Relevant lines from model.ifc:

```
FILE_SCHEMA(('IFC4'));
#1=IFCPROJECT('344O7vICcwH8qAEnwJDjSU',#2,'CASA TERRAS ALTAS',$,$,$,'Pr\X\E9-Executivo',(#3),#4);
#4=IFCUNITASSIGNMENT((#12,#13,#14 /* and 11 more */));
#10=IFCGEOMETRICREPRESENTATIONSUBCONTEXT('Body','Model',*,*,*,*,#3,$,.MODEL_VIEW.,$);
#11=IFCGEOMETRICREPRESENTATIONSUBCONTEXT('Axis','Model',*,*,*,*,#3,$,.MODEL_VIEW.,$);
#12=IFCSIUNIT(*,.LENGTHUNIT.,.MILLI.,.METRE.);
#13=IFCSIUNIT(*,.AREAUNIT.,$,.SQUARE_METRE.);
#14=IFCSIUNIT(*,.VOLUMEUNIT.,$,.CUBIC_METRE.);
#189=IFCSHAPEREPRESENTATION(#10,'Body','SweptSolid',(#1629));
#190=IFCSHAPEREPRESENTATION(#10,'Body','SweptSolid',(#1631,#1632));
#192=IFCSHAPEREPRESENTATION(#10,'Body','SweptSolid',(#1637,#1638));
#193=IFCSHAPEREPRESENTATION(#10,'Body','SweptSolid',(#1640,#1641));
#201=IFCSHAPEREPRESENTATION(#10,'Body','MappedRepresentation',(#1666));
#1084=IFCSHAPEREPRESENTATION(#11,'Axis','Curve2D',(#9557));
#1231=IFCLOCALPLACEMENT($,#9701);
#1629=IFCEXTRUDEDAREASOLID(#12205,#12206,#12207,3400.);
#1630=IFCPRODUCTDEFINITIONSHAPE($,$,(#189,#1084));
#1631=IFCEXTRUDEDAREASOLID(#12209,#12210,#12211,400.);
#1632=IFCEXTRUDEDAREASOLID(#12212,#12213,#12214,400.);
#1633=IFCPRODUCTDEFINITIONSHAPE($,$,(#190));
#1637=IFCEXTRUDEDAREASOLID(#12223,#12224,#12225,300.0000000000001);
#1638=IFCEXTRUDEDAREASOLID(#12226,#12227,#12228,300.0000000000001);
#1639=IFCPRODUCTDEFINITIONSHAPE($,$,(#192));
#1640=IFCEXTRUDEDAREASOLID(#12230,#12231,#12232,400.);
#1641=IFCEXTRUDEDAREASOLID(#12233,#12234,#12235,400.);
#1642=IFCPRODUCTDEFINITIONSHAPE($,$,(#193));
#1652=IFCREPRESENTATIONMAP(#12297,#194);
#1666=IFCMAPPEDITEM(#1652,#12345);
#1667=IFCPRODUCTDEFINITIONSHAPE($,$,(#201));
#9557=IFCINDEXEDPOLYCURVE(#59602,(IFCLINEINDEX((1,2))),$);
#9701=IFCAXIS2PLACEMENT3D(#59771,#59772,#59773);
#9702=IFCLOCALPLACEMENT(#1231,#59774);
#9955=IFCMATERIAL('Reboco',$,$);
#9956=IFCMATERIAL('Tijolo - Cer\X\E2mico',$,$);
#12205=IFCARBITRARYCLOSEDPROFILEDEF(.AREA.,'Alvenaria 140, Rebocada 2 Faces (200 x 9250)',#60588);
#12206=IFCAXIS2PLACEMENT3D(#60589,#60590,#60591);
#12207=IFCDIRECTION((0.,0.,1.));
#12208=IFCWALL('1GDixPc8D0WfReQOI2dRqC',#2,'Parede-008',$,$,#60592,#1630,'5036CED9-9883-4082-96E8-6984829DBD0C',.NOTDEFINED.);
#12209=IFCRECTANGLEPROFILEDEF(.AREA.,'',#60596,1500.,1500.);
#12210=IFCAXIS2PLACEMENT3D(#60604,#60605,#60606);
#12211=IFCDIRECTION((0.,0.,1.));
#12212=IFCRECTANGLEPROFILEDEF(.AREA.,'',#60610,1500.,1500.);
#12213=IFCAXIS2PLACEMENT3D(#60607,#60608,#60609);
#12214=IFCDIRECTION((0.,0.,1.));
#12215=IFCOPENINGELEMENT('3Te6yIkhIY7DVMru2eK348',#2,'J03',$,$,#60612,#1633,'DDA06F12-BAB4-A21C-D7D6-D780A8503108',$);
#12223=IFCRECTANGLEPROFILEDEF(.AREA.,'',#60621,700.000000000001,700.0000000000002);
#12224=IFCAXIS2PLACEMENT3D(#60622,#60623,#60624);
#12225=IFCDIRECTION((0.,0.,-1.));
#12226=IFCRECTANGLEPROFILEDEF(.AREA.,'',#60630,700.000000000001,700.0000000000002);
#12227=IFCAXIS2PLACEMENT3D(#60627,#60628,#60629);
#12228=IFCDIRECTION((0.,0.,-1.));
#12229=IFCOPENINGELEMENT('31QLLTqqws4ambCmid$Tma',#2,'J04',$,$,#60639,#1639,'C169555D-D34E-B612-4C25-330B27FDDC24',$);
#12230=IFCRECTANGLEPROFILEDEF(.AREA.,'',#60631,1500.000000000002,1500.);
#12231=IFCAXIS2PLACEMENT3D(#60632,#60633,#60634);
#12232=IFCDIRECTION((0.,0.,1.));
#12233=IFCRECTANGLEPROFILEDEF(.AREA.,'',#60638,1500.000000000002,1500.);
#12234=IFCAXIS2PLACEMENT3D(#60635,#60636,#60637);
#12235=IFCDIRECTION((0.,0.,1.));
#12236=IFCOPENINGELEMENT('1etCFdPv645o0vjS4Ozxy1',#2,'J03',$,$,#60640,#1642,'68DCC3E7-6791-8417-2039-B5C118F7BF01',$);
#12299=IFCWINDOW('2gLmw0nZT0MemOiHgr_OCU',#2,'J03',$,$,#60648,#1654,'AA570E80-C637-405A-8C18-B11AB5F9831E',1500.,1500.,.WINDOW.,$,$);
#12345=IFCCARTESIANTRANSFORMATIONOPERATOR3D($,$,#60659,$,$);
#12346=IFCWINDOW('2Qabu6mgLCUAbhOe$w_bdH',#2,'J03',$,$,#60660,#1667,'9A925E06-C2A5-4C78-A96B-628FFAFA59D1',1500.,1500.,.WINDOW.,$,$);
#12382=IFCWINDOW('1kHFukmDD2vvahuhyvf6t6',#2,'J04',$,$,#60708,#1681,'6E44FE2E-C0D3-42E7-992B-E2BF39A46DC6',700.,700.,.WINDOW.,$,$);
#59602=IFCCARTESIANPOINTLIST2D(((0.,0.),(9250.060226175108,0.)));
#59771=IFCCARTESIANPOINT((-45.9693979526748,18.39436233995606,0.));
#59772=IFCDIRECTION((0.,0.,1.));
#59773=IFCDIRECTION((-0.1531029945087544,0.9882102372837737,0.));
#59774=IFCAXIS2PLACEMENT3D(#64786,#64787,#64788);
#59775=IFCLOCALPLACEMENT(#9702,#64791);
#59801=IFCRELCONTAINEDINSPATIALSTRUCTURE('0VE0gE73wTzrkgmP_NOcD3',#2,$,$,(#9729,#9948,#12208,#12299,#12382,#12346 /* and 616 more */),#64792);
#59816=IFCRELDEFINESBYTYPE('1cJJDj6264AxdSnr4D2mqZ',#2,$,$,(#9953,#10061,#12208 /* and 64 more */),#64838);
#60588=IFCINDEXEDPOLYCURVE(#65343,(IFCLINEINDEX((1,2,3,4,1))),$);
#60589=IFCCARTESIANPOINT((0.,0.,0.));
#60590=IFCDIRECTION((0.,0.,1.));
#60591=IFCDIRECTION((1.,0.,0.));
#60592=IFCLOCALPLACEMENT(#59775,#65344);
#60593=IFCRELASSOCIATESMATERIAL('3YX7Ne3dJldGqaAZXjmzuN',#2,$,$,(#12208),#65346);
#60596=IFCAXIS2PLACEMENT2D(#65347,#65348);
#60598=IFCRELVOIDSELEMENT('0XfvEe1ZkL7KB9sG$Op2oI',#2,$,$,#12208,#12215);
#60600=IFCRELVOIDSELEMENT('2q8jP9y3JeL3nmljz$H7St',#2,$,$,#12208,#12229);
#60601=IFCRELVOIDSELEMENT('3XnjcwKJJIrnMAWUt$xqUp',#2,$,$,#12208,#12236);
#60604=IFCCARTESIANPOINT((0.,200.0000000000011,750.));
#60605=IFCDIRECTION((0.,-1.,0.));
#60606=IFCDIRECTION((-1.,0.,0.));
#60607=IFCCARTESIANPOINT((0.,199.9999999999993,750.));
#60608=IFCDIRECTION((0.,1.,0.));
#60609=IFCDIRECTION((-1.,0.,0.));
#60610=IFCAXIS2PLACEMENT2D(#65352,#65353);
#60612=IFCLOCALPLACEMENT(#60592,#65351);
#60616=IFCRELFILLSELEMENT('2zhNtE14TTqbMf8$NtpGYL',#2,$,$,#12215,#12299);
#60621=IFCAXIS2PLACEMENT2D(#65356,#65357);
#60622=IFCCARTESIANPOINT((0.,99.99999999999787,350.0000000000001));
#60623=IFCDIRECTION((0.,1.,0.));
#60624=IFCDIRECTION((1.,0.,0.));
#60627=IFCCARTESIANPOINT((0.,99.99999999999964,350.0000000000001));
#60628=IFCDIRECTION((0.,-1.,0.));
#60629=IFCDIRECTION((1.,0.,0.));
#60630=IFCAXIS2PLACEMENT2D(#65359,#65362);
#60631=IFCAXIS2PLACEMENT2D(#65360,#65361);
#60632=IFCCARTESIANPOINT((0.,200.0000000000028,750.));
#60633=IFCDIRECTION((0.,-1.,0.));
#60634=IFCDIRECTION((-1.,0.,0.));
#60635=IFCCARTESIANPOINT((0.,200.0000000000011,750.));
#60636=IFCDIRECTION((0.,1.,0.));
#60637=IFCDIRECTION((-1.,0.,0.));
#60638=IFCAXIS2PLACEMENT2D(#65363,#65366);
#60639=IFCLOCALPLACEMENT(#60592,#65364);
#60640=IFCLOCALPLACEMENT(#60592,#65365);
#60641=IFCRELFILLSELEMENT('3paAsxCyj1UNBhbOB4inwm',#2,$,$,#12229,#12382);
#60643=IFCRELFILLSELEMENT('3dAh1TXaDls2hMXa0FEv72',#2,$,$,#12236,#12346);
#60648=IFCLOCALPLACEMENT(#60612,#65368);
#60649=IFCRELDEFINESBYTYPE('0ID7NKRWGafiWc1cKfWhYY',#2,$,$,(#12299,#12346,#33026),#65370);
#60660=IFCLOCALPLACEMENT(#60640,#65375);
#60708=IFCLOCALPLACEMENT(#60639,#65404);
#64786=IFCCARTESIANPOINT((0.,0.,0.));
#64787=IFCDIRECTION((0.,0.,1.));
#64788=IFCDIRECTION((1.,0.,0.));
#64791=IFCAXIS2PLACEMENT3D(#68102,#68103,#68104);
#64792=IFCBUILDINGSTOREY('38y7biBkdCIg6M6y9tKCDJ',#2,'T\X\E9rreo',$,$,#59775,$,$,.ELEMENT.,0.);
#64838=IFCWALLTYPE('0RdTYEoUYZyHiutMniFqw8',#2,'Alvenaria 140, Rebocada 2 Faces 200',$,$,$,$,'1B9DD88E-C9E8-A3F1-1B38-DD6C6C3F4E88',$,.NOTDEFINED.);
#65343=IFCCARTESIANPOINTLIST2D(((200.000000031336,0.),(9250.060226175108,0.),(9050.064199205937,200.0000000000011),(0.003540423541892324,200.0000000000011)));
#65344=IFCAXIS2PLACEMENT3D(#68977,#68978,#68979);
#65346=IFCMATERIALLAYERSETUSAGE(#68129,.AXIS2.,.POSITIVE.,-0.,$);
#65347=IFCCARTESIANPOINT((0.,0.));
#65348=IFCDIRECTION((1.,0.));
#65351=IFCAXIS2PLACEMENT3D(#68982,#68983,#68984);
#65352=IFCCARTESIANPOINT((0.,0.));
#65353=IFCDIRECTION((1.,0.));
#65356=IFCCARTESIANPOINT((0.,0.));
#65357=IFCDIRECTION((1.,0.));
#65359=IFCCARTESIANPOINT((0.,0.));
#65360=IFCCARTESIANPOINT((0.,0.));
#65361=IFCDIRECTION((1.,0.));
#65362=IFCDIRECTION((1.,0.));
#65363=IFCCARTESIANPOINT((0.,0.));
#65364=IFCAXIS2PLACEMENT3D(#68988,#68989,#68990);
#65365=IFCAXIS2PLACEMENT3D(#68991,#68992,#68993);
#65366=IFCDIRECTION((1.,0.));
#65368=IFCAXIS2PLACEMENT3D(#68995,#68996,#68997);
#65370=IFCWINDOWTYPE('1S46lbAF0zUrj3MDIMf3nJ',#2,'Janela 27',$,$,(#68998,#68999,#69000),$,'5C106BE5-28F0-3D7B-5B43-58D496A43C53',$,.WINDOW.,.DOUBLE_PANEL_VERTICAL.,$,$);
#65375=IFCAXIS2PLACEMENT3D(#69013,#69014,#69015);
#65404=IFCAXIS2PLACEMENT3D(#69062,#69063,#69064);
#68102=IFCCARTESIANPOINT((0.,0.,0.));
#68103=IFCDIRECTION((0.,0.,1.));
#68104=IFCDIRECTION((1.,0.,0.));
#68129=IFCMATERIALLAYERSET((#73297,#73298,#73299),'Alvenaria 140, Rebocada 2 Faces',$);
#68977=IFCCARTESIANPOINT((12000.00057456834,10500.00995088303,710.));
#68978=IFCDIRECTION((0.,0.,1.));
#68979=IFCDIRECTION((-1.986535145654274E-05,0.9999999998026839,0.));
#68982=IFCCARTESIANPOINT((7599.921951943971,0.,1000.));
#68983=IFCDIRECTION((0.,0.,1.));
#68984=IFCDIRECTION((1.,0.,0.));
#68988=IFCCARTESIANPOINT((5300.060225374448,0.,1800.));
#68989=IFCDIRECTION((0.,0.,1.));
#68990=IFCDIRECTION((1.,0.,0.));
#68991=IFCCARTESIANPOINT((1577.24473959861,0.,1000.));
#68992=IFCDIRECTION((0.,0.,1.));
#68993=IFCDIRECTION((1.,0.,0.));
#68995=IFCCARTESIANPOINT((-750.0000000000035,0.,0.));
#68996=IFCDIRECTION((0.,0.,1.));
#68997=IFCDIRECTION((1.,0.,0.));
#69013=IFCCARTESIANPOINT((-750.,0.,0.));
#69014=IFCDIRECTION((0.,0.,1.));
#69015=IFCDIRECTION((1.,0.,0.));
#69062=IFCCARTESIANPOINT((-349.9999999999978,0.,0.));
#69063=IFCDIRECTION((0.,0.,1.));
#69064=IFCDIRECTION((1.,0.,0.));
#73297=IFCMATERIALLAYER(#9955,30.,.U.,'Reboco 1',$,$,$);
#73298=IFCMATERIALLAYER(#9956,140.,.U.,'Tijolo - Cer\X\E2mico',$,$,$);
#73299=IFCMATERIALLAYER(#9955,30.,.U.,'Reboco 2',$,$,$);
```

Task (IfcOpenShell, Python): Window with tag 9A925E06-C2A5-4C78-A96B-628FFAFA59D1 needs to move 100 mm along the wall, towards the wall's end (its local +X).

```python
import ifcopenshell
import ifcopenshell.api.geometry
import ifcopenshell.util.placement
import ifcopenshell.util.unit

model = ifcopenshell.open("model.ifc")
unit_scale = ifcopenshell.util.unit.calculate_unit_scale(model)

window = model.by_guid("2Qabu6mgLCUAbhOe$w_bdH")
opening = window.FillsVoids[0].RelatingOpeningElement
wall = opening.VoidsElements[0].RelatingBuildingElement

wall_matrix = ifcopenshell.util.placement.get_local_placement(wall.ObjectPlacement)
shift = wall_matrix[:3, 0] * 0.1 / unit_scale
before = ifcopenshell.util.placement.get_local_placement(window.ObjectPlacement)[:3, 3].copy()

# The window is placed relative to its opening, so it follows when the opening moves.
matrix = ifcopenshell.util.placement.get_local_placement(opening.ObjectPlacement)
matrix[:3, 3] += shift
ifcopenshell.api.geometry.edit_object_placement(
    model, product=opening, matrix=matrix, is_si=False, should_transform_children=True
)

after = ifcopenshell.util.placement.get_local_placement(window.ObjectPlacement)[:3, 3]
print("window moved by", (after - before).round(3) + 0.0)

model.write("model_updated.ifc")
```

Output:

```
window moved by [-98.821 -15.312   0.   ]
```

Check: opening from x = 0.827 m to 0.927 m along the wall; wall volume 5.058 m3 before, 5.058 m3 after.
